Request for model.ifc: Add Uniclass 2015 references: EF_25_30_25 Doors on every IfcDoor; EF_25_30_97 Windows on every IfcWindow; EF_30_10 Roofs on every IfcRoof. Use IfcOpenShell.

First a look at what the model holds.

```python
import ifcopenshell

model = ifcopenshell.open("model.ifc")
print(model.schema)
print("classifications:", [c.Name for c in model.by_type("IfcClassification")])
for ifc_class in ("IfcDoor", "IfcRoof", "IfcStair", "IfcWall", "IfcWindow"):
    print(ifc_class, len(model.by_type(ifc_class)))
```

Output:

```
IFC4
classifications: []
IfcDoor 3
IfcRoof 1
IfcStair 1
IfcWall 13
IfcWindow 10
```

```python
import ifcopenshell
import ifcopenshell.api.classification

model = ifcopenshell.open("model.ifc")

system = ifcopenshell.api.classification.add_classification(model, classification="Uniclass 2015")

codes = {
    "IfcDoor": ("EF_25_30_25", "Doors"),
    "IfcWindow": ("EF_25_30_97", "Windows"),
    "IfcRoof": ("EF_30_10", "Roofs"),
}
for ifc_class, (code, name) in codes.items():
    products = model.by_type(ifc_class)
    ifcopenshell.api.classification.add_reference(
        model, products=products, classification=system, identification=code, name=name
    )
    print(code, len(products))

model.write("model_edited.ifc")
```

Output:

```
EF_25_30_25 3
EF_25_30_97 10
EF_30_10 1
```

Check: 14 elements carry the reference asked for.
